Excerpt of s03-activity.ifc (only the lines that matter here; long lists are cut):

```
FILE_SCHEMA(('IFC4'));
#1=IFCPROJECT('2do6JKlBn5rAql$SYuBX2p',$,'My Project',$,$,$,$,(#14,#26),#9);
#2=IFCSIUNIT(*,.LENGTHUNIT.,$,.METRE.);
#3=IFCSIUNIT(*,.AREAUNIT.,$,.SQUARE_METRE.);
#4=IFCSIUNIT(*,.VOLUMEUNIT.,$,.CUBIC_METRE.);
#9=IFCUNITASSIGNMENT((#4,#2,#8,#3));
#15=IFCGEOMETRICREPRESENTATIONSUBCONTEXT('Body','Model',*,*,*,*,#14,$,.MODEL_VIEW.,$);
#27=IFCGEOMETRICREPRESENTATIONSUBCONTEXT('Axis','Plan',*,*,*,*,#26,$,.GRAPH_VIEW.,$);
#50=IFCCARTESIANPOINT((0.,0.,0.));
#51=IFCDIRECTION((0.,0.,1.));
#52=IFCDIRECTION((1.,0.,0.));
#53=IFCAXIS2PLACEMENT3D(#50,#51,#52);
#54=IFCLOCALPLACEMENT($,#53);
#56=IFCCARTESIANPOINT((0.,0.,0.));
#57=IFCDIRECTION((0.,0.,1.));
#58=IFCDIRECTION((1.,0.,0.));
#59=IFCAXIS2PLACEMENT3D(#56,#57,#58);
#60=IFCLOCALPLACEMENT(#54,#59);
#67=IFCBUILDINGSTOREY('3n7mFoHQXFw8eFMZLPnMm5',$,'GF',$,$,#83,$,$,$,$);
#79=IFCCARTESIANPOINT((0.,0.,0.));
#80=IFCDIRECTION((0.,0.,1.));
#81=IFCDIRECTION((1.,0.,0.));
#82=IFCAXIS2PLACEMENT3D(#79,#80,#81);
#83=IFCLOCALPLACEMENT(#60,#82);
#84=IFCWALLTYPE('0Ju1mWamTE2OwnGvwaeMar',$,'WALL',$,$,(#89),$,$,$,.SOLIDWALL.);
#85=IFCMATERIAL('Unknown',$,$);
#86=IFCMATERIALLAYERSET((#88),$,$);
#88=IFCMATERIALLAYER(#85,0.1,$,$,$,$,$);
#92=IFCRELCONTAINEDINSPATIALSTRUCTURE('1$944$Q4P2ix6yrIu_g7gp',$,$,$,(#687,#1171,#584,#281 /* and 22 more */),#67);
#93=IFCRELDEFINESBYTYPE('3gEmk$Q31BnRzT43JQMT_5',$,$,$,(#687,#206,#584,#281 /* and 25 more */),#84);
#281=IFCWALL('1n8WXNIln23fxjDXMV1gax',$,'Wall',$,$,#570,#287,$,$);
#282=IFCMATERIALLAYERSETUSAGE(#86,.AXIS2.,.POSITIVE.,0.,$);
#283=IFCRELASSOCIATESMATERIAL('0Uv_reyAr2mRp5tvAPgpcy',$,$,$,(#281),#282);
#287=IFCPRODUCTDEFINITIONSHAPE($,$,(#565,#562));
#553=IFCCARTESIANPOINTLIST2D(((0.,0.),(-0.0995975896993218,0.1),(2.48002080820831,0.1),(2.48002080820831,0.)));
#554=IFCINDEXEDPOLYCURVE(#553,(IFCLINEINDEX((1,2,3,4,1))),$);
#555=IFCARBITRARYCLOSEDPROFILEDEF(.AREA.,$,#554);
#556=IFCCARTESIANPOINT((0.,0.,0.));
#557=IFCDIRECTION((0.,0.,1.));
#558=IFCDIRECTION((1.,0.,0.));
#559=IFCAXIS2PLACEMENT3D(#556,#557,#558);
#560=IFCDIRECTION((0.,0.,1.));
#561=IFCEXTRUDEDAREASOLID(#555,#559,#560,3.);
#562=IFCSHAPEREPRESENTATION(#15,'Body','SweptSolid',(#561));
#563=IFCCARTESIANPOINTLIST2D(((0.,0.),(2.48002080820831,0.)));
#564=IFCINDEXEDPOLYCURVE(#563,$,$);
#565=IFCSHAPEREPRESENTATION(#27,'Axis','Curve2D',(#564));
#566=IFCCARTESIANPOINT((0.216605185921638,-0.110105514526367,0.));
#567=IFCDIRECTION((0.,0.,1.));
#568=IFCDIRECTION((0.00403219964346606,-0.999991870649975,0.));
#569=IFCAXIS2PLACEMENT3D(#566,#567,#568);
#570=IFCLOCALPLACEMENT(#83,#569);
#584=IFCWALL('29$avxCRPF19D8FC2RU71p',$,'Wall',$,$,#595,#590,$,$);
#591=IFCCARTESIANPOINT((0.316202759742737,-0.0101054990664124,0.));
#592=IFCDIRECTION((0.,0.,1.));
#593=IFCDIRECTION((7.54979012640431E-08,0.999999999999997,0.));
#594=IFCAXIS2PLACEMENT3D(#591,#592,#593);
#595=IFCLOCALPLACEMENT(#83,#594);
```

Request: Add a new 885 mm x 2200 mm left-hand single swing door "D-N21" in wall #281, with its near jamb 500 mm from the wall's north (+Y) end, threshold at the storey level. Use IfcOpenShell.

```python
import numpy as np
import ifcopenshell
import ifcopenshell.api.feature
import ifcopenshell.api.geometry
import ifcopenshell.api.root
import ifcopenshell.api.spatial
import ifcopenshell.geom
import ifcopenshell.util.element
import ifcopenshell.util.placement
import ifcopenshell.util.representation
import ifcopenshell.util.shape
import ifcopenshell.util.unit

model = ifcopenshell.open("s03-activity.ifc")
unit_scale = ifcopenshell.util.unit.calculate_unit_scale(model)
settings = ifcopenshell.geom.settings()


def volume(element):
    """Net volume in cubic metres, openings subtracted."""
    shape = ifcopenshell.geom.create_shape(settings, element)
    return ifcopenshell.util.shape.get_volume(shape.geometry)


wall = model.by_guid("1n8WXNIln23fxjDXMV1gax")
storey = ifcopenshell.util.element.get_container(wall, ifc_class="IfcBuildingStorey")
context = ifcopenshell.util.representation.get_context(model, "Model", "Body", "MODEL_VIEW")
before = volume(wall)

width, height, from_end, sill = 0.885, 2.2, 0.5, 0.0  # metres

# The wall runs along its own X axis, and the end named is its -X end.
wall_shape = ifcopenshell.geom.create_shape(settings, wall)
x, y, z = ifcopenshell.util.shape.get_vertices(wall_shape.geometry).T
start = x.min() + from_end
face, thickness = float(y.min()), float(y.max() - y.min())
wall_matrix = ifcopenshell.util.placement.get_local_placement(wall.ObjectPlacement)
level = ifcopenshell.util.placement.get_local_placement(storey.ObjectPlacement)[2, 3]


def in_wall(x, y):
    """Placement at x, y metres in the wall's axes, at sill height."""
    matrix = wall_matrix.copy()
    matrix[:, 3] = wall_matrix @ np.array([x / unit_scale, y / unit_scale, 0.0, 1.0])
    matrix[2, 3] = level + sill / unit_scale
    return matrix


# Opening: a box that overshoots both wall faces by 50 mm.
opening = ifcopenshell.api.root.create_entity(model, ifc_class="IfcOpeningElement", predefined_type="OPENING")
box = ifcopenshell.api.geometry.add_wall_representation(
    model, context=context, length=width, height=height, thickness=thickness + 0.1
)
ifcopenshell.api.geometry.assign_representation(model, product=opening, representation=box)
ifcopenshell.api.geometry.edit_object_placement(model, product=opening, matrix=in_wall(start, face - 0.05), is_si=False)
ifcopenshell.api.feature.add_feature(model, feature=opening, element=wall)

door = ifcopenshell.api.root.create_entity(model, ifc_class="IfcDoor", name="D-N21", predefined_type="DOOR")
door.OverallWidth, door.OverallHeight = width / unit_scale, height / unit_scale
door.OperationType = "SINGLE_SWING_LEFT"
body = ifcopenshell.api.geometry.add_door_representation(
    model,
    context=context,
    overall_width=door.OverallWidth,
    overall_height=door.OverallHeight,
    operation_type="SINGLE_SWING_LEFT",
    lining_properties={"LiningDepth": thickness / unit_scale, "ThresholdDepth": thickness / unit_scale},
)
ifcopenshell.api.geometry.assign_representation(model, product=door, representation=body)
ifcopenshell.api.spatial.assign_container(model, products=[door], relating_structure=storey)
ifcopenshell.api.feature.add_filling(model, opening=opening, element=door)

# The lining spans the wall, so the door starts at the wall face.
ifcopenshell.api.geometry.edit_object_placement(model, product=door, matrix=in_wall(start, face), is_si=False)

after = volume(wall)

print(f"wall volume {before:.3f} -> {after:.3f} m3")

model.write("s03-activity_updated.ifc")
```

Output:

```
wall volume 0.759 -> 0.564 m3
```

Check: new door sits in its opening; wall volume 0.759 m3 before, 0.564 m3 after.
